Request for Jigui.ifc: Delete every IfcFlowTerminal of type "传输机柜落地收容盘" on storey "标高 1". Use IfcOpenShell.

First a look at what the model holds.

```python
import ifcopenshell
import ifcopenshell.util.element

model = ifcopenshell.open("Jigui.ifc")
print(model.schema)
storey = next(s for s in model.by_type("IfcBuildingStorey") if s.Name == "标高 1")
terminals = [e for e in ifcopenshell.util.element.get_decomposition(storey) if e.is_a("IfcFlowTerminal")]
seen = {}
for e in terminals:
    element_type = ifcopenshell.util.element.get_type(e)
    name = element_type.Name if element_type not in (None, e) else None
    seen[name] = seen.get(name, 0) + 1
for name, count in sorted(seen.items(), key=str):
    print(count, "x", name)
```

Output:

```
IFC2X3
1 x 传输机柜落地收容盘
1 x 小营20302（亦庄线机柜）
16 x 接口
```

```python
import ifcopenshell
import ifcopenshell.api.root
import ifcopenshell.util.element

model = ifcopenshell.open("Jigui.ifc")

storey = next(s for s in model.by_type("IfcBuildingStorey") if s.Name == "标高 1")
terminals = [e for e in ifcopenshell.util.element.get_decomposition(storey) if e.is_a("IfcFlowTerminal")]
targets = [e for e in terminals if (t := ifcopenshell.util.element.get_type(e)) not in (None, e) and t.Name == "传输机柜落地收容盘"]

for e in targets:
    ifcopenshell.api.root.remove_product(model, product=e)
print(len(targets), "removed")

model.write("Jigui_updated.ifc")
```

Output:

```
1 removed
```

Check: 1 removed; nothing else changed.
